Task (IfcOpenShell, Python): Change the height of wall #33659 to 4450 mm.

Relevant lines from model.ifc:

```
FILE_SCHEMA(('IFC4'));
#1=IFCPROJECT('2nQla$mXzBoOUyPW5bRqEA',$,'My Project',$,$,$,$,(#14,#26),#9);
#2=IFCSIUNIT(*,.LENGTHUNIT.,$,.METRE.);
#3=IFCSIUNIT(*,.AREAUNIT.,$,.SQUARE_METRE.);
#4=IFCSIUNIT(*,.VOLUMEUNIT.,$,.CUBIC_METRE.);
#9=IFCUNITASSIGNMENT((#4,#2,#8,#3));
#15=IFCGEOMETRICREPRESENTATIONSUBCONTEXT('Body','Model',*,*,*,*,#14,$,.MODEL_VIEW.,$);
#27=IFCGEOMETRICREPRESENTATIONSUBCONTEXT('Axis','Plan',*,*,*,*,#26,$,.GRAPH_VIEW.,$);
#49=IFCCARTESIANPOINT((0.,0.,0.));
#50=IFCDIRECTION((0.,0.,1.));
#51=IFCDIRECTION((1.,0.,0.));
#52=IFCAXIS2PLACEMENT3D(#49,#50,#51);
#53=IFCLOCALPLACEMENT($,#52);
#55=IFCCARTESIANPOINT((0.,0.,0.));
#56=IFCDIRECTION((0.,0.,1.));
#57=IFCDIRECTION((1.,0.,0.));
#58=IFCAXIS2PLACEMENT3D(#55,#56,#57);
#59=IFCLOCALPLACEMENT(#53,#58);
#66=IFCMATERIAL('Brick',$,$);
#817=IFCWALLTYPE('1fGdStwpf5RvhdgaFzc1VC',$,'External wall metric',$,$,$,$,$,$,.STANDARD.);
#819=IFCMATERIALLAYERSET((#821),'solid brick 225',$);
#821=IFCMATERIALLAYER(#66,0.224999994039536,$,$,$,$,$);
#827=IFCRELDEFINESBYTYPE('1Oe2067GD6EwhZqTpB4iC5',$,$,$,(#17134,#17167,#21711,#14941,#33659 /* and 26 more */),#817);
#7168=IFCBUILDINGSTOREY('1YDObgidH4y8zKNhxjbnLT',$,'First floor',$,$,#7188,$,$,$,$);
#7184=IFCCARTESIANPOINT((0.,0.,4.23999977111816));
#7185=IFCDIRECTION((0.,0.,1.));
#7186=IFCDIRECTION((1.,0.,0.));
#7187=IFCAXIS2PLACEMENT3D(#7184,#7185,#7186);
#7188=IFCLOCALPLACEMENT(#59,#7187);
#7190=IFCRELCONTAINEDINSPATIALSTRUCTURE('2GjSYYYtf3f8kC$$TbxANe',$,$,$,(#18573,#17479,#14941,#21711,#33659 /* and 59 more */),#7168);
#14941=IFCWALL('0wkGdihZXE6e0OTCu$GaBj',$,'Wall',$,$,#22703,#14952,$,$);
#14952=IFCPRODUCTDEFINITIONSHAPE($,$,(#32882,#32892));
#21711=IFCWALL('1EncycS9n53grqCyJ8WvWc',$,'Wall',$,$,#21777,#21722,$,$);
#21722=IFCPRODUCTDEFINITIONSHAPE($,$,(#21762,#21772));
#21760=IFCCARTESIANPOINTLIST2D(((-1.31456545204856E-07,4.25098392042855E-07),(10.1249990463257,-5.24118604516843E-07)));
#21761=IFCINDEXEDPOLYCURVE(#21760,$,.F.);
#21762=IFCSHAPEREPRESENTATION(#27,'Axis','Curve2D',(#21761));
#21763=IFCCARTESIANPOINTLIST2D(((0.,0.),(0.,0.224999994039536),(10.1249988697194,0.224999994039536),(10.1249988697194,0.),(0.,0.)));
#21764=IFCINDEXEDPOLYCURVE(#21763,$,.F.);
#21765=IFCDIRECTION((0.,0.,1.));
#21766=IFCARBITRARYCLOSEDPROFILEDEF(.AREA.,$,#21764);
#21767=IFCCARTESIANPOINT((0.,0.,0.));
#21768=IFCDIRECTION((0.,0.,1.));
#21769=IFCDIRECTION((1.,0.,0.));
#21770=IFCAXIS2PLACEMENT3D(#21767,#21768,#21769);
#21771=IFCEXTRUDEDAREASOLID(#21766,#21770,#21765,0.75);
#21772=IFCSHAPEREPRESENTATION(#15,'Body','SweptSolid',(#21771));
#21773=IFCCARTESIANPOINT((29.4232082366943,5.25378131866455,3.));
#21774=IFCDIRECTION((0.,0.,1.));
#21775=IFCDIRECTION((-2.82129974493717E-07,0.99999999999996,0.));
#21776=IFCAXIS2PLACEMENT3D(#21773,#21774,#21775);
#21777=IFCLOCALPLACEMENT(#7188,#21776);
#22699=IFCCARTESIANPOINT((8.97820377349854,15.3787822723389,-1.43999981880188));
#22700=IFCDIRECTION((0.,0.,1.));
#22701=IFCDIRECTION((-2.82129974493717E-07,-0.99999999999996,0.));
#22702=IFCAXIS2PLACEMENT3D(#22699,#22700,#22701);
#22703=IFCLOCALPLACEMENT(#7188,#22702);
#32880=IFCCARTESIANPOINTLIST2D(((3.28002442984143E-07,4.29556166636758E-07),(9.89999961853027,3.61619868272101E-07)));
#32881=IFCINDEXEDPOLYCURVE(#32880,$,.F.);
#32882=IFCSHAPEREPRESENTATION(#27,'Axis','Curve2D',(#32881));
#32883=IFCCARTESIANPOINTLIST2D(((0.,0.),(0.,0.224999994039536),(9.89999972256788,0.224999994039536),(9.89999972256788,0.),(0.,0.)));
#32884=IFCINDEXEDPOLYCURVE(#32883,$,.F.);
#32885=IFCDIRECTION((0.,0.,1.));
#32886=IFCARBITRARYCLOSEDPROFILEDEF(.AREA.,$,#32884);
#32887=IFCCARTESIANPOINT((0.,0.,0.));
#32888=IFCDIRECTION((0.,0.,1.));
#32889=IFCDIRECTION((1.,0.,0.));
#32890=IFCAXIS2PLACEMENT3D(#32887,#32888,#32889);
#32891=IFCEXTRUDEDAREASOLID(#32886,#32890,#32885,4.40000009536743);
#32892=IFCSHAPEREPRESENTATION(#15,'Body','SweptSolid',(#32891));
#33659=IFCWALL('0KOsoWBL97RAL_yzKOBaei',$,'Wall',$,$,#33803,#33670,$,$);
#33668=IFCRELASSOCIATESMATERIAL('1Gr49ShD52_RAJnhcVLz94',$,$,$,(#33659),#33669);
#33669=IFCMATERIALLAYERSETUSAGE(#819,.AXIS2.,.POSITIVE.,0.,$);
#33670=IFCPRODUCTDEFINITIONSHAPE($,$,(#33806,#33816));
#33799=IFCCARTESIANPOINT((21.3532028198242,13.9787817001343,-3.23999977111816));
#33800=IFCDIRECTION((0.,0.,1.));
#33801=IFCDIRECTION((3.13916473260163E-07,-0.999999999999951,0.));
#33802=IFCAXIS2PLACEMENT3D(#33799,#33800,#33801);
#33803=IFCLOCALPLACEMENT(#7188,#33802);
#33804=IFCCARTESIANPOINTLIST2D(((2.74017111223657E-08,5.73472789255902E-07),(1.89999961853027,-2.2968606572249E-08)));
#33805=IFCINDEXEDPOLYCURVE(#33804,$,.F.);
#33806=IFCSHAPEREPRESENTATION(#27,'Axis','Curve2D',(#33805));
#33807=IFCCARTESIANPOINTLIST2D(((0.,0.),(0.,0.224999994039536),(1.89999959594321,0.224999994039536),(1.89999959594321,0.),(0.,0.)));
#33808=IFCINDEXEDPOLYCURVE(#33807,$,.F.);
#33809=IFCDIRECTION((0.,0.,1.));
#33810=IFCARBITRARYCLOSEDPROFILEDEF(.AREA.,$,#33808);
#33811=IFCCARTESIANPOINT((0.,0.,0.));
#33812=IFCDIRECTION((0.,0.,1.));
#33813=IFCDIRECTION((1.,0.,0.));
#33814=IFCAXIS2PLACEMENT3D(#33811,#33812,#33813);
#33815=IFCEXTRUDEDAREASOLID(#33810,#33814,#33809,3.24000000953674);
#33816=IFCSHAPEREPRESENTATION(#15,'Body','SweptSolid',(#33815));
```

```python
import ifcopenshell
import ifcopenshell.geom
import ifcopenshell.util.representation
import ifcopenshell.util.shape

model = ifcopenshell.open("model.ifc")
settings = ifcopenshell.geom.settings()


def volume(element):
    """Net volume in cubic metres, openings subtracted."""
    shape = ifcopenshell.geom.create_shape(settings, element)
    return ifcopenshell.util.shape.get_volume(shape.geometry)


wall = model.by_guid("0KOsoWBL97RAL_yzKOBaei")
before = volume(wall)

body = ifcopenshell.util.representation.get_representation(wall, "Model", "Body")
solid = body.Items[0]
old_height = solid.Depth
solid.Depth = 4.45
after = volume(wall)

print(f"height {old_height:g} -> {solid.Depth:g}, volume {before:.3f} -> {after:.3f} m3")

model.write("model_edited.ifc")
```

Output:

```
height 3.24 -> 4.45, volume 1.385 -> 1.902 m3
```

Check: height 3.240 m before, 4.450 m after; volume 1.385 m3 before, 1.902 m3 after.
